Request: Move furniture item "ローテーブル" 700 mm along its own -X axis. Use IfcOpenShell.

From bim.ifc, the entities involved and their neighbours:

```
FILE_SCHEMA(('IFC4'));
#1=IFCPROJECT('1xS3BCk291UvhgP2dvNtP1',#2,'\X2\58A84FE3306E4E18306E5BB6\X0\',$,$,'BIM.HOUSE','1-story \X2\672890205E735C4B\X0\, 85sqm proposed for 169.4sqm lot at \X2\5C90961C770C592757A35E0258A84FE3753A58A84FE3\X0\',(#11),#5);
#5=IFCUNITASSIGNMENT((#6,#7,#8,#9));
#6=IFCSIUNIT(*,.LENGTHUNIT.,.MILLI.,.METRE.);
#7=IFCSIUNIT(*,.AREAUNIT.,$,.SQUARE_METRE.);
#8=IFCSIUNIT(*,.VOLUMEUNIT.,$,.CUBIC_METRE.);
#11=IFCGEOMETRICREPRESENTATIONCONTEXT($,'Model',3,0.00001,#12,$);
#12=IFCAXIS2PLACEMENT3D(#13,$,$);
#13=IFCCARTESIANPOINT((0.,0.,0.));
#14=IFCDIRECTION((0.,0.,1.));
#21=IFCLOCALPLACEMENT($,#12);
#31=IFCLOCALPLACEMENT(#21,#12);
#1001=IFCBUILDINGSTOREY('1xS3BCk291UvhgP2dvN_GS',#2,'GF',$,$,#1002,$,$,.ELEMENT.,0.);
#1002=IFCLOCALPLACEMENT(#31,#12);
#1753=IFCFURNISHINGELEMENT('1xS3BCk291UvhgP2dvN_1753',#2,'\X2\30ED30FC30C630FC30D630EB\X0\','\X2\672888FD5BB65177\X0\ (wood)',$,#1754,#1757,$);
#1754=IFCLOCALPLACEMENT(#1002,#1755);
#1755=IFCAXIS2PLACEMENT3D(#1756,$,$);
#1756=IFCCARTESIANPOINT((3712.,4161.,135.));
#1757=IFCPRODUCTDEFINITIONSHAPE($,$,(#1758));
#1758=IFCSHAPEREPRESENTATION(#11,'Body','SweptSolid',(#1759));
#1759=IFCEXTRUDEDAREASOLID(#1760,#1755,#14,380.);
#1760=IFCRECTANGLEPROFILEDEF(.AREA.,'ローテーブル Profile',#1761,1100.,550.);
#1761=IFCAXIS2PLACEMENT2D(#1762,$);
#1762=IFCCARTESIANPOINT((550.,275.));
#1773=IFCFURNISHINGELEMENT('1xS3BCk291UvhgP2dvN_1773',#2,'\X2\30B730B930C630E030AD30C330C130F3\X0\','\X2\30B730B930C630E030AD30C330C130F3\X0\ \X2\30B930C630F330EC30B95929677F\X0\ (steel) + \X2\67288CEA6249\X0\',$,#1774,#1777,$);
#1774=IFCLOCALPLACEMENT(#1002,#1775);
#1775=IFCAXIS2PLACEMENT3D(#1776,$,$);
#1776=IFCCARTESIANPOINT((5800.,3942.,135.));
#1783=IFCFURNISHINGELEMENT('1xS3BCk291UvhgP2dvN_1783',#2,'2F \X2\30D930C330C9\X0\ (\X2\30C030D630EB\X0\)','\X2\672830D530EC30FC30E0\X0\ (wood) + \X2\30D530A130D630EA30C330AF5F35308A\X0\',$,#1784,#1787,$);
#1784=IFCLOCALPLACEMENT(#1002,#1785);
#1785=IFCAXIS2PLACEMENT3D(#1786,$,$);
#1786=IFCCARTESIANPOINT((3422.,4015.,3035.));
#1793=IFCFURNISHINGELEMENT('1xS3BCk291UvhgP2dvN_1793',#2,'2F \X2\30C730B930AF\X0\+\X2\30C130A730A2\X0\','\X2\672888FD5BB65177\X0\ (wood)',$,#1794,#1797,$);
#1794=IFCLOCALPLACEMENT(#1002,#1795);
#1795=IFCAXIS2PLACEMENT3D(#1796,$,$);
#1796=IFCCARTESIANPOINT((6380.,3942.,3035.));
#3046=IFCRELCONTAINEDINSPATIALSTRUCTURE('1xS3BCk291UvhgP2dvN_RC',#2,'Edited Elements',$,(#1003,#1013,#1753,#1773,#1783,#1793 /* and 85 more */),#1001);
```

```python
import ifcopenshell
import ifcopenshell.api.geometry
import ifcopenshell.util.placement

model = ifcopenshell.open("bim.ifc")

item = model.by_guid("1xS3BCk291UvhgP2dvN_1753")
matrix = ifcopenshell.util.placement.get_local_placement(item.ObjectPlacement)
matrix[:3, 3] -= matrix[:3, 0] * 700.0
ifcopenshell.api.geometry.edit_object_placement(model, product=item, matrix=matrix, is_si=False)

print(ifcopenshell.util.placement.get_local_placement(item.ObjectPlacement).round(3) + 0.0)

model.write("bim_rev.ifc")
```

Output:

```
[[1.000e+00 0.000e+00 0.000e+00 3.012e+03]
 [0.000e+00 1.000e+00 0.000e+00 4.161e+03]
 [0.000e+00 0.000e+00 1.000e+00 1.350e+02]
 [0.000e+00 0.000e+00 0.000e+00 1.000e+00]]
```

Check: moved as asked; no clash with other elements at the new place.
